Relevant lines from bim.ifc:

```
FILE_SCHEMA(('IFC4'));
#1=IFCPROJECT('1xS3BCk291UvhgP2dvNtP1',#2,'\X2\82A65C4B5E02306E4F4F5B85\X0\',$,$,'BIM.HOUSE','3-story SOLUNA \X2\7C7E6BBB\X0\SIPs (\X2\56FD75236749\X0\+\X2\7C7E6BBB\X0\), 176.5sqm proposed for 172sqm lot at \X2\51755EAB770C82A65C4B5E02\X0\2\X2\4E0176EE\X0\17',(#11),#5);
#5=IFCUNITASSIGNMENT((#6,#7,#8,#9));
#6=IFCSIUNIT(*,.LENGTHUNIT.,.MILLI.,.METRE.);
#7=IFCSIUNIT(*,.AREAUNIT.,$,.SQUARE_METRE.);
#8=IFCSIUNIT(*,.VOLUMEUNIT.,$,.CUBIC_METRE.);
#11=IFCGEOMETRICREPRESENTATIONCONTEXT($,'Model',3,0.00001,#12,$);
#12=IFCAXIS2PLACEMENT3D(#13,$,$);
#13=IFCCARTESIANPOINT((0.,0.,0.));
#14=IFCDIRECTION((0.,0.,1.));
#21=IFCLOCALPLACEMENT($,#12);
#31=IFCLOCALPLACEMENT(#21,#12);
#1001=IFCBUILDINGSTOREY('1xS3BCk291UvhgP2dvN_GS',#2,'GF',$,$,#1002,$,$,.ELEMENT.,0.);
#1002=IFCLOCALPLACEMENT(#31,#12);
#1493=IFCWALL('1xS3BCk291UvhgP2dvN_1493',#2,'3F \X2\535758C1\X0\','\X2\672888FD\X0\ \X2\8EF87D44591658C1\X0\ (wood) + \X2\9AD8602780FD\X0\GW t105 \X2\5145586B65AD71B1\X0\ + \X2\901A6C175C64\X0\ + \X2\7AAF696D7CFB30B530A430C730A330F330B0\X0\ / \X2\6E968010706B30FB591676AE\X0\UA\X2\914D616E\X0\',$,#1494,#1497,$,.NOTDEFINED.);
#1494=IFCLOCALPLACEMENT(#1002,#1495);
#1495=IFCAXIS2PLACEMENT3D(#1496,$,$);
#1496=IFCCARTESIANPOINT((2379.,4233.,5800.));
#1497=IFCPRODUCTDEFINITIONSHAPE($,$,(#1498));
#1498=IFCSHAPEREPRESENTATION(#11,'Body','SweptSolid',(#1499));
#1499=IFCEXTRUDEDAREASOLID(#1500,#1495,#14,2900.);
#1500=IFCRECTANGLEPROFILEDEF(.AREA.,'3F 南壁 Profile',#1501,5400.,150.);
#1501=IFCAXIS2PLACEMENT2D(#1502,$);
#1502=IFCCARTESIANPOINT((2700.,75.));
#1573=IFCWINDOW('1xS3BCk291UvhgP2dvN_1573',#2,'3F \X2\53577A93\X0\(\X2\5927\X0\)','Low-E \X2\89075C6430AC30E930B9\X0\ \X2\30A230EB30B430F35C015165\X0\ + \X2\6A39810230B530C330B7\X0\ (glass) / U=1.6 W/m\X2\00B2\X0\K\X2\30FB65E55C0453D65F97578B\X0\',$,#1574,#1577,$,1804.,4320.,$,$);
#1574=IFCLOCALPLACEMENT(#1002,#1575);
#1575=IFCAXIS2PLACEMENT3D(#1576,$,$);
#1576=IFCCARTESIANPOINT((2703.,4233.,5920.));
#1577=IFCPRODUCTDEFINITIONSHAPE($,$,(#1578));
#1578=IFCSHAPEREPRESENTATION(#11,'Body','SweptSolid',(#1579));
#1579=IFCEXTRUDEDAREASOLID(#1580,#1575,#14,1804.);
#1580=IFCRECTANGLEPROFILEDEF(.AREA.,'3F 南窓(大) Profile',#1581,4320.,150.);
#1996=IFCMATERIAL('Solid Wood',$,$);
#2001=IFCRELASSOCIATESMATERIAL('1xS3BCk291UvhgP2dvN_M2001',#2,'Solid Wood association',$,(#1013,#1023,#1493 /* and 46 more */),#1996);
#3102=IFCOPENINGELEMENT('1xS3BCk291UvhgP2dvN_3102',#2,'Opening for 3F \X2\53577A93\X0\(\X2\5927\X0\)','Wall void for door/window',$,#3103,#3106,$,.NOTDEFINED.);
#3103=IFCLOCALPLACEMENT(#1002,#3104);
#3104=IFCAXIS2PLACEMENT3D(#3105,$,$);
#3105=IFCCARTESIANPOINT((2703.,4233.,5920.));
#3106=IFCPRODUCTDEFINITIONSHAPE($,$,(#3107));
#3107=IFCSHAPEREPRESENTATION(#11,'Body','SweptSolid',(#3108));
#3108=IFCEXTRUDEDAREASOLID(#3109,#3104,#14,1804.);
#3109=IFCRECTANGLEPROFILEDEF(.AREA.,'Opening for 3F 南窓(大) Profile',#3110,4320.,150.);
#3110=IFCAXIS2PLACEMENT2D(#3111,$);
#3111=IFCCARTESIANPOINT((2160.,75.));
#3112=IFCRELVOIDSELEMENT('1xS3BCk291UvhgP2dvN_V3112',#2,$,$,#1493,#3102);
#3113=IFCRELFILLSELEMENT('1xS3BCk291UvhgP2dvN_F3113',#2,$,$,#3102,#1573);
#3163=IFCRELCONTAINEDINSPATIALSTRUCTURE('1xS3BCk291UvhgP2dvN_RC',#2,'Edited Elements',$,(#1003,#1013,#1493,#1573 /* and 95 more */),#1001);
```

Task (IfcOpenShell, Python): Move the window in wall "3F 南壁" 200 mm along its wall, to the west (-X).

```python
import ifcopenshell
import ifcopenshell.api.geometry
import ifcopenshell.util.placement

model = ifcopenshell.open("bim.ifc")

window = model.by_guid("1xS3BCk291UvhgP2dvN_1573")
opening = window.FillsVoids[0].RelatingOpeningElement
wall = opening.VoidsElements[0].RelatingBuildingElement

wall_matrix = ifcopenshell.util.placement.get_local_placement(wall.ObjectPlacement)
shift = wall_matrix[:3, 0] * -200.0
before = ifcopenshell.util.placement.get_local_placement(window.ObjectPlacement)[:3, 3].copy()

# The window is not placed relative to its opening, so move both.
for product in (opening, window):
    matrix = ifcopenshell.util.placement.get_local_placement(product.ObjectPlacement)
    matrix[:3, 3] += shift
    ifcopenshell.api.geometry.edit_object_placement(model, product=product, matrix=matrix, is_si=False)

after = ifcopenshell.util.placement.get_local_placement(window.ObjectPlacement)[:3, 3]
print("window moved by", (after - before).round(3) + 0.0)

model.write("bim_edited.ifc")
```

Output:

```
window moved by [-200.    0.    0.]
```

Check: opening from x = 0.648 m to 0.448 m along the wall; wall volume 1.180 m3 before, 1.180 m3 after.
